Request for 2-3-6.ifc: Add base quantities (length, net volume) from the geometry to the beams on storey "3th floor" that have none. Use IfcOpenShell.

First a look at what the model holds.

```python
import ifcopenshell
import ifcopenshell.util.element
import ifcopenshell.util.unit

model = ifcopenshell.open("2-3-6.ifc")
print(model.schema)
for unit_type in ("LENGTHUNIT", "AREAUNIT", "VOLUMEUNIT"):
    print(unit_type, ifcopenshell.util.unit.calculate_unit_scale(model, unit_type))
storey = next(s for s in model.by_type("IfcBuildingStorey") if s.Name == "3th floor")
beams = [e for e in ifcopenshell.util.element.get_decomposition(storey) if e.is_a("IfcBeam")]
for e in sorted(beams, key=lambda e: e.id()):
    print(e.id(), e.is_a(), e.Name, list(ifcopenshell.util.element.get_psets(e, qtos_only=True)), sep=" | ")
```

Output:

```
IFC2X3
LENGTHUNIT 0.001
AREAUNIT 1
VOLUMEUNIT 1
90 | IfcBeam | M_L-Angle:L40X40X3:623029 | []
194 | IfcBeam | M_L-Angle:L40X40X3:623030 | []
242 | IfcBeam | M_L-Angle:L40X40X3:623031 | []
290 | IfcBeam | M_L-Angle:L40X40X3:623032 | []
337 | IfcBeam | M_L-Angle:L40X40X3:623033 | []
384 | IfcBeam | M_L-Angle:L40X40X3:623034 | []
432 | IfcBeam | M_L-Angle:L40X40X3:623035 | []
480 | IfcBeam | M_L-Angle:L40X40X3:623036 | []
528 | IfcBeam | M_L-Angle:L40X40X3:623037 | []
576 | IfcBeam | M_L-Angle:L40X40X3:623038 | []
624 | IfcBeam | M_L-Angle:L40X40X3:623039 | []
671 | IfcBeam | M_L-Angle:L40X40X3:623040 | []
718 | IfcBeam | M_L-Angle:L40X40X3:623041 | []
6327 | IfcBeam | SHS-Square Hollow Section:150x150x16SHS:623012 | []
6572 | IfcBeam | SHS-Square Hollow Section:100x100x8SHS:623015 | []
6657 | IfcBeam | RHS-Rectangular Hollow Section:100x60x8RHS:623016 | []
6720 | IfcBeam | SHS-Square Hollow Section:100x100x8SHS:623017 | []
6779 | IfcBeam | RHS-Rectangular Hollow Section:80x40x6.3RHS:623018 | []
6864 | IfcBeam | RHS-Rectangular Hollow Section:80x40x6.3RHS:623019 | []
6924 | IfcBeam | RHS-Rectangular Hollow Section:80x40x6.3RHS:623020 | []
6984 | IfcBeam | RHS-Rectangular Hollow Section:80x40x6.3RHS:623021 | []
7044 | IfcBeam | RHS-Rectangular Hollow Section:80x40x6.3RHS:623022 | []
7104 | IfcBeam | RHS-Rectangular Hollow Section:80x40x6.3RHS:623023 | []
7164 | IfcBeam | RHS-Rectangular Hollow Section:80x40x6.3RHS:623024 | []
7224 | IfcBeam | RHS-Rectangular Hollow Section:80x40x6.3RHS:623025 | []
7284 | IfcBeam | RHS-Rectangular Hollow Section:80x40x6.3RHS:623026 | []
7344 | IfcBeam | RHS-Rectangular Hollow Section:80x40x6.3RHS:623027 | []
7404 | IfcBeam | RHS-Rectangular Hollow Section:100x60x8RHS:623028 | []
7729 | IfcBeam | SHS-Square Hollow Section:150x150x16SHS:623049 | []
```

```python
import ifcopenshell
import ifcopenshell.api.pset
import ifcopenshell.geom
import ifcopenshell.util.element
import ifcopenshell.util.shape
import ifcopenshell.util.unit

model = ifcopenshell.open("2-3-6.ifc")
unit_scale = ifcopenshell.util.unit.calculate_unit_scale(model)
volume_scale = ifcopenshell.util.unit.calculate_unit_scale(model, "VOLUMEUNIT")
settings = ifcopenshell.geom.settings()

storey = next(s for s in model.by_type("IfcBuildingStorey") if s.Name == "3th floor")
beams = [e for e in ifcopenshell.util.element.get_decomposition(storey) if e.is_a("IfcBeam")]

for e in sorted(beams, key=lambda e: e.id()):
    if ifcopenshell.util.element.get_psets(e, qtos_only=True, should_inherit=False):
        continue
    # Geometry comes back in metres, in the element's own axes.
    shape = ifcopenshell.geom.create_shape(settings, e)
    values = {
        "Length": ifcopenshell.util.shape.get_max_xyz(shape.geometry) / unit_scale,
        "NetVolume": ifcopenshell.util.shape.get_volume(shape.geometry) / volume_scale,
    }
    qto = ifcopenshell.api.pset.add_qto(model, product=e, name="BaseQuantities")
    ifcopenshell.api.pset.edit_qto(model, qto=qto, properties=values)
    print(e.id(), {k: round(v, 3) for k, v in values.items()})

model.write("2-3-6_edited.ifc")
```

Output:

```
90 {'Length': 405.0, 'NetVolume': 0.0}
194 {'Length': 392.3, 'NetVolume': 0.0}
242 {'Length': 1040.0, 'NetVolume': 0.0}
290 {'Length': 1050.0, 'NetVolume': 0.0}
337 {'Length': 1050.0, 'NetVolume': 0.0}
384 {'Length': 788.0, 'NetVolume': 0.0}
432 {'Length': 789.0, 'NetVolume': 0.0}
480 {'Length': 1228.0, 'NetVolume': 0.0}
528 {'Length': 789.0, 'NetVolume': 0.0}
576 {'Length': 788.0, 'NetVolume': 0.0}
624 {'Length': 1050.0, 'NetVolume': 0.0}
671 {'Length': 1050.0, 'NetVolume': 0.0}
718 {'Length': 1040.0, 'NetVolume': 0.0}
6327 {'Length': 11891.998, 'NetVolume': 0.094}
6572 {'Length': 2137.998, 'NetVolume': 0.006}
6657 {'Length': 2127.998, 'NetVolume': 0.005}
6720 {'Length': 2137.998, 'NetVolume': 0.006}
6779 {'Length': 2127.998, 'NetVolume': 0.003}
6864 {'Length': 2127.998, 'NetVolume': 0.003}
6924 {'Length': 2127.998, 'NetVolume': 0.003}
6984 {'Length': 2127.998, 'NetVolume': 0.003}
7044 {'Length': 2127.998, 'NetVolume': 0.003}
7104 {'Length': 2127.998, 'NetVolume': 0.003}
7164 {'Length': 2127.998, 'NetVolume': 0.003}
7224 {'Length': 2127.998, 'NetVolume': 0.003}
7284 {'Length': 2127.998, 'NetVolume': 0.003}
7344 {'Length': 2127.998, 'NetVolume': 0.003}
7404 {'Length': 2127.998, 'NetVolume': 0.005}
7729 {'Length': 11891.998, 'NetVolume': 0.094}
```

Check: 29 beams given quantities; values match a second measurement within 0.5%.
